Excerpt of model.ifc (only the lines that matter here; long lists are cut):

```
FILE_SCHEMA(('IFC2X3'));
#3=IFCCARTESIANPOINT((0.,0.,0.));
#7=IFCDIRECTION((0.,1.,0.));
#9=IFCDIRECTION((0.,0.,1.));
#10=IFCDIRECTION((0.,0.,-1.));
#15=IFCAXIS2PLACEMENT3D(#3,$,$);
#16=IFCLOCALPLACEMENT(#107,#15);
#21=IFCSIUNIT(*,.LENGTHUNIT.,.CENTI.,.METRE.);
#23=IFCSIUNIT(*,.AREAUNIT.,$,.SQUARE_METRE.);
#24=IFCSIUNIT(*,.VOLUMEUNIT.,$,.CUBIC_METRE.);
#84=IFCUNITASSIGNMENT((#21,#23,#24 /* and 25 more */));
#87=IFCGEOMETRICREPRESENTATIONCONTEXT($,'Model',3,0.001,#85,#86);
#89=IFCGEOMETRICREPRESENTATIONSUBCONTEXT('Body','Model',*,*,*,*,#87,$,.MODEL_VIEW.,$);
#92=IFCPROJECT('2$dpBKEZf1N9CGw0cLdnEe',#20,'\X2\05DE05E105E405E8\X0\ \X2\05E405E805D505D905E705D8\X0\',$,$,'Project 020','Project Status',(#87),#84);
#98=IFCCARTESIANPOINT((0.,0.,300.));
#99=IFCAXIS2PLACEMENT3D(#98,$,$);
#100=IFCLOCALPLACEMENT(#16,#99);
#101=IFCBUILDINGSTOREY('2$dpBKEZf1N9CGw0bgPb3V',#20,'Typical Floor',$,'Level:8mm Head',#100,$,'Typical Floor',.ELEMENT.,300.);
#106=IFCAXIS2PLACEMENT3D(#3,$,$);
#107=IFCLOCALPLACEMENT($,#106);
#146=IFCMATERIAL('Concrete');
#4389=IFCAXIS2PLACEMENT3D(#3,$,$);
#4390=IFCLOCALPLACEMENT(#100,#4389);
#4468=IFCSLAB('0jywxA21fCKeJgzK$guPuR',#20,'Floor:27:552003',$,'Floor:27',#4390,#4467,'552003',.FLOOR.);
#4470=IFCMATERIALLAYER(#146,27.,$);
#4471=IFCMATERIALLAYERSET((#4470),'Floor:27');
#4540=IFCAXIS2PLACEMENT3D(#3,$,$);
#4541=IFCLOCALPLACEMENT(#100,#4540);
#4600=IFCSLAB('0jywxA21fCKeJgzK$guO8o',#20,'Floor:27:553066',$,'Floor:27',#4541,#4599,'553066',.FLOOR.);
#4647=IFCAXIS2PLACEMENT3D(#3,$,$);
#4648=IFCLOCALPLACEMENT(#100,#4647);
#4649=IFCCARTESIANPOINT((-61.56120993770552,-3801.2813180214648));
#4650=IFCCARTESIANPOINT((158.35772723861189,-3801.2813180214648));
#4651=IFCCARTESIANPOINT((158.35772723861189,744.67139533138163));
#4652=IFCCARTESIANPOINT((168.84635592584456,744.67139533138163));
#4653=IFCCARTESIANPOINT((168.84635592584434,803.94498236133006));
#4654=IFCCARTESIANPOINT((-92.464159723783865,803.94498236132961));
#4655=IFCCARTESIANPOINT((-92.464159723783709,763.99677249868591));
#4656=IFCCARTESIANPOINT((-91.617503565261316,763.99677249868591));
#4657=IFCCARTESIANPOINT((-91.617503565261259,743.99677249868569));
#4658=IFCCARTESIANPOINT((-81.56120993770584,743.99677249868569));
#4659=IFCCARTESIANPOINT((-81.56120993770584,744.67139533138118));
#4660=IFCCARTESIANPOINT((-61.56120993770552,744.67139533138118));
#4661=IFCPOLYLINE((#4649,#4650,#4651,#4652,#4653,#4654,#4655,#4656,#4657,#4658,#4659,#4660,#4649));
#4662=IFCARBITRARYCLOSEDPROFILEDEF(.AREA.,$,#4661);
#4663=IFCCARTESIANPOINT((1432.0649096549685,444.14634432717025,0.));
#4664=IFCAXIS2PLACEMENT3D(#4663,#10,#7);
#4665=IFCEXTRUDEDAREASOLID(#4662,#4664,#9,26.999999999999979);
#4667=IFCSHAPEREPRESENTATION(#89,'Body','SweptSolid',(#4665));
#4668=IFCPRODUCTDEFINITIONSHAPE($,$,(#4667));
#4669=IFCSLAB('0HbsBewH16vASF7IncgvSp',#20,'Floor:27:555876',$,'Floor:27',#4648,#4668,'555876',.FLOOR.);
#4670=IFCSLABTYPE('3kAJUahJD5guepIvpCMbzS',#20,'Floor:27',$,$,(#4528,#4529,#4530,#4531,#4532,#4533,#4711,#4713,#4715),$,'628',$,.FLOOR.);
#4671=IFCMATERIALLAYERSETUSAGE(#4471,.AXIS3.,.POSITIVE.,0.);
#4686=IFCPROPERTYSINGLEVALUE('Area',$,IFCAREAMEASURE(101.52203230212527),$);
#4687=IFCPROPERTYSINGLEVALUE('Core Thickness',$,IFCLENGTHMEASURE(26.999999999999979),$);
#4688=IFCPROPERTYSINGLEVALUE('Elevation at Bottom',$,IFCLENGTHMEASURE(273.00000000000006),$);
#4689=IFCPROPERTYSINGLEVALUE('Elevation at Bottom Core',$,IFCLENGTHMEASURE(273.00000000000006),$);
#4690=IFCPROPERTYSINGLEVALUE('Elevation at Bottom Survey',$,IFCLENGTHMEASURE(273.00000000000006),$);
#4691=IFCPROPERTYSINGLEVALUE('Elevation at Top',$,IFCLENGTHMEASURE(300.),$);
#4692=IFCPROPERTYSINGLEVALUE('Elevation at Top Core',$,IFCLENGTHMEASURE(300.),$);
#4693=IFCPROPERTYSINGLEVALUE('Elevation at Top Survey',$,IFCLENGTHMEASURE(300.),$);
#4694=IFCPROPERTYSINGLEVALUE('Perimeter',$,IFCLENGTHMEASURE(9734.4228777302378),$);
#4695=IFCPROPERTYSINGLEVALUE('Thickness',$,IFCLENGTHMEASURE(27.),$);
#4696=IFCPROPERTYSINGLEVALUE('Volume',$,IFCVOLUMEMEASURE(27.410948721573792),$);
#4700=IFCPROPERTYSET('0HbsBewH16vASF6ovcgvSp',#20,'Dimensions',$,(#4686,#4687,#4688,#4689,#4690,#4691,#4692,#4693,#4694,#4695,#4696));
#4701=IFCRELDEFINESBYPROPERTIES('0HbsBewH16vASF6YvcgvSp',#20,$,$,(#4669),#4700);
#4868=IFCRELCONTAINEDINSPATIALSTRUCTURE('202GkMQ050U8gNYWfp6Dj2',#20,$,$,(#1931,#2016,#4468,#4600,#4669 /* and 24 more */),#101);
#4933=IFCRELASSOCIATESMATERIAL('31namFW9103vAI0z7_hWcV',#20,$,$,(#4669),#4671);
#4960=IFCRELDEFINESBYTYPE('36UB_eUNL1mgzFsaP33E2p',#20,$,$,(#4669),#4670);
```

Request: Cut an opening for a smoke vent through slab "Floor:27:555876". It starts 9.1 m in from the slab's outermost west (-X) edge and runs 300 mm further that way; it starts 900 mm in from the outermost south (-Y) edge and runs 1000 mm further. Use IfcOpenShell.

```python
import numpy as np
import ifcopenshell
import ifcopenshell.api.feature
import ifcopenshell.api.geometry
import ifcopenshell.api.pset
import ifcopenshell.api.root
import ifcopenshell.geom
import ifcopenshell.util.element
import ifcopenshell.util.placement
import ifcopenshell.util.representation
import ifcopenshell.util.shape
import ifcopenshell.util.unit

model = ifcopenshell.open("model.ifc")
unit_scale = ifcopenshell.util.unit.calculate_unit_scale(model)
area_scale = ifcopenshell.util.unit.calculate_unit_scale(model, "AREAUNIT")
volume_scale = ifcopenshell.util.unit.calculate_unit_scale(model, "VOLUMEUNIT")
settings = ifcopenshell.geom.settings()


def volume(element):
    """Net volume in cubic metres, openings subtracted."""
    shape = ifcopenshell.geom.create_shape(settings, element)
    return ifcopenshell.util.shape.get_volume(shape.geometry)


slab = model.by_guid("0HbsBewH16vASF7IncgvSp")
before = volume(slab)

# Extent in the slab's own axes, in metres. The edges named are its -X and -Y sides.
slab_shape = ifcopenshell.geom.create_shape(settings, slab)
vertices = ifcopenshell.util.shape.get_vertices(slab_shape.geometry)
x_min, y_min, bottom = vertices.min(axis=0)
top = vertices[:, 2].max()

opening = ifcopenshell.api.root.create_entity(model, ifc_class="IfcOpeningElement", name="Smoke vent opening")
context = ifcopenshell.util.representation.get_context(model, "Model", "Body", "MODEL_VIEW")
width, depth = 0.3, 1
outline = [(0.0, 0.0), (width, 0.0), (width, depth), (0.0, depth), (0.0, 0.0)]
# Overshoot both faces by 50 mm so the cut is clean.
shape = ifcopenshell.api.geometry.add_slab_representation(
    model, context=context, depth=top - bottom + 0.1, polyline=outline
)
ifcopenshell.api.geometry.assign_representation(model, product=opening, representation=shape)

matrix = ifcopenshell.util.placement.get_local_placement(slab.ObjectPlacement)
matrix[:, 3] = matrix @ np.append(np.array([x_min + 9.1, y_min + 0.9, bottom - 0.05]) / unit_scale, 1.0)
ifcopenshell.api.geometry.edit_object_placement(model, product=opening, matrix=matrix, is_si=False)
ifcopenshell.api.feature.add_feature(model, feature=opening, element=slab)

after = volume(slab)

# Update the slab's stored quantities.
pset = model.by_id(ifcopenshell.util.element.get_pset(slab, "Dimensions", should_inherit=False)["id"])
ifcopenshell.api.pset.edit_pset(model, pset=pset, properties={
    "Area": model.create_entity("IfcAreaMeasure", after / (top - bottom) / area_scale),
    "Volume": model.create_entity("IfcVolumeMeasure", after / volume_scale),
})

print(f"slab volume {before:.3f} -> {after:.3f} m3")

model.write("model-out.ifc")
```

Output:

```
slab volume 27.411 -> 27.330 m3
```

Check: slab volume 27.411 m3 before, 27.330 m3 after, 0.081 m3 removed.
